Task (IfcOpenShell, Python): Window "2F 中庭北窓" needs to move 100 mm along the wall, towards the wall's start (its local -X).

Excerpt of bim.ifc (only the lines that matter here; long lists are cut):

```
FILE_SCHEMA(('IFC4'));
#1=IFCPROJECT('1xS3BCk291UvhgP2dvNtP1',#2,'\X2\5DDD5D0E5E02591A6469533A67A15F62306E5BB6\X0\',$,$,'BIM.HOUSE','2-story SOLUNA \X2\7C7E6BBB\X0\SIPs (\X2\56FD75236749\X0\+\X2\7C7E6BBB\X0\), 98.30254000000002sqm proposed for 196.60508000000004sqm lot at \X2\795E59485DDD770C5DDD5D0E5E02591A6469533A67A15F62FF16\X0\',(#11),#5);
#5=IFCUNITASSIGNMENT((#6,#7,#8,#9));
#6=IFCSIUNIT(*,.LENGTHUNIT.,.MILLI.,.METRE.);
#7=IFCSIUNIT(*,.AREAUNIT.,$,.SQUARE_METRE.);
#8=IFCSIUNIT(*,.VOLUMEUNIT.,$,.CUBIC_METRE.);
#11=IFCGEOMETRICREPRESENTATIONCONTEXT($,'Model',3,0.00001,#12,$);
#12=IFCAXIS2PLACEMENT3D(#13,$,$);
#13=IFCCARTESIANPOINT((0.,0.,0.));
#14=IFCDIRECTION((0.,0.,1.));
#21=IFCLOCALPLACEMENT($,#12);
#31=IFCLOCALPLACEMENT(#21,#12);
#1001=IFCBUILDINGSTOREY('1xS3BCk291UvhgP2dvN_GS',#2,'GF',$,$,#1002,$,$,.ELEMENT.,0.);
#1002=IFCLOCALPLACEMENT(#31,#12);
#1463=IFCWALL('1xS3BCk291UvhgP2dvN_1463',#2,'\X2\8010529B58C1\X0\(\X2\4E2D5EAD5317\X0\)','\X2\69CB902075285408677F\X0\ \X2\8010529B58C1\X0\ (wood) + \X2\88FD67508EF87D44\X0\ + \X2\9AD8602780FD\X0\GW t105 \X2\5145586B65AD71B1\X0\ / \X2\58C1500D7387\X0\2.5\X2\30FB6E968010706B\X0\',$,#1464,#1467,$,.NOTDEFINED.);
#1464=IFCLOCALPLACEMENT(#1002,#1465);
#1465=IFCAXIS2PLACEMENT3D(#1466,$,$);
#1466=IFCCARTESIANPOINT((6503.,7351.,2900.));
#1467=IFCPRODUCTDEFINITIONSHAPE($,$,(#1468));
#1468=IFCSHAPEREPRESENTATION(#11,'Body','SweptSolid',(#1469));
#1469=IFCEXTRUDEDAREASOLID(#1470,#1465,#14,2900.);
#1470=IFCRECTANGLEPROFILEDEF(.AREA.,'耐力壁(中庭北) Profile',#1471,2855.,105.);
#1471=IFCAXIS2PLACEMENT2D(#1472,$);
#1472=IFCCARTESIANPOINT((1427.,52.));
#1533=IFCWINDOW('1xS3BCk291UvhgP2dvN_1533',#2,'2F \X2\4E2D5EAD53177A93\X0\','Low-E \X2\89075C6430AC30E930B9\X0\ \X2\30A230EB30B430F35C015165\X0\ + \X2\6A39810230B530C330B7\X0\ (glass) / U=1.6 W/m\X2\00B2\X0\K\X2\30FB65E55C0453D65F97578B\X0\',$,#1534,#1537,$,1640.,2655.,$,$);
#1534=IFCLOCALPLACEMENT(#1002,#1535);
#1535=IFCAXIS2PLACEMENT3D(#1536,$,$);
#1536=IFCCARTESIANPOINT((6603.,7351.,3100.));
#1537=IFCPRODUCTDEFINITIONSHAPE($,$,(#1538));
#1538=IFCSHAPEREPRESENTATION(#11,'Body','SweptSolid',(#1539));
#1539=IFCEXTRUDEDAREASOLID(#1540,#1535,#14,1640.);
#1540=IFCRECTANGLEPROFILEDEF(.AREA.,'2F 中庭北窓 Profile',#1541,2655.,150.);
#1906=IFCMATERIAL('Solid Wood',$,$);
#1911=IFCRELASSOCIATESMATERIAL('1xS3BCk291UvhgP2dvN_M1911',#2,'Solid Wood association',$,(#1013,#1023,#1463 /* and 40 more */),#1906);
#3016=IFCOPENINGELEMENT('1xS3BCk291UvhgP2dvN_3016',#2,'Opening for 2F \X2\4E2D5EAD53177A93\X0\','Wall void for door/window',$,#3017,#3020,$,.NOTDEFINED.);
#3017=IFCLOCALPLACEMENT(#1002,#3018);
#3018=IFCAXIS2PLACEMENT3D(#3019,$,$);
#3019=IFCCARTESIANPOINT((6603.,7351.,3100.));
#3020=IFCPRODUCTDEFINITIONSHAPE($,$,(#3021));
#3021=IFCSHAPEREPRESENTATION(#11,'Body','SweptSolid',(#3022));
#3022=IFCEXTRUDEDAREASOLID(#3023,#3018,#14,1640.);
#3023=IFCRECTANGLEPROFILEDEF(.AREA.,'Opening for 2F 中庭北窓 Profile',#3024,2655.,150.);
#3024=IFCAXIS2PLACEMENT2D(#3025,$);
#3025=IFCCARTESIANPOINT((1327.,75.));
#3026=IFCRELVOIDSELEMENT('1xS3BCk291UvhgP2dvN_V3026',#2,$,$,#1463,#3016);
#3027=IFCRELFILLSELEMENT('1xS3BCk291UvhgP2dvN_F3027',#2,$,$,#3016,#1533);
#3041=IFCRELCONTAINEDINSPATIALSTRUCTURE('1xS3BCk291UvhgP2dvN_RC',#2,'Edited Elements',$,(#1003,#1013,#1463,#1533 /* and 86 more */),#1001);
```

```python
import ifcopenshell
import ifcopenshell.api.geometry
import ifcopenshell.util.placement

model = ifcopenshell.open("bim.ifc")

window = model.by_guid("1xS3BCk291UvhgP2dvN_1533")
opening = window.FillsVoids[0].RelatingOpeningElement
wall = opening.VoidsElements[0].RelatingBuildingElement

wall_matrix = ifcopenshell.util.placement.get_local_placement(wall.ObjectPlacement)
shift = wall_matrix[:3, 0] * -100.0
before = ifcopenshell.util.placement.get_local_placement(window.ObjectPlacement)[:3, 3].copy()

# The window is not placed relative to its opening, so move both.
for product in (opening, window):
    matrix = ifcopenshell.util.placement.get_local_placement(product.ObjectPlacement)
    matrix[:3, 3] += shift
    ifcopenshell.api.geometry.edit_object_placement(model, product=product, matrix=matrix, is_si=False)

after = ifcopenshell.util.placement.get_local_placement(window.ObjectPlacement)[:3, 3]
print("window moved by", (after - before).round(3) + 0.0)

model.write("bim_v2.ifc")
```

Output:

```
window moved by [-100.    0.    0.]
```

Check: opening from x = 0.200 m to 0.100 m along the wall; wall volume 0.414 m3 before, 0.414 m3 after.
